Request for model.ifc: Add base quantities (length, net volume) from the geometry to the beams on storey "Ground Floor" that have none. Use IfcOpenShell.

First a look at what the model holds.

```python
import ifcopenshell
import ifcopenshell.util.element
import ifcopenshell.util.unit

model = ifcopenshell.open("model.ifc")
print(model.schema)
for unit_type in ("LENGTHUNIT", "AREAUNIT", "VOLUMEUNIT"):
    print(unit_type, ifcopenshell.util.unit.calculate_unit_scale(model, unit_type))
storey = next(s for s in model.by_type("IfcBuildingStorey") if s.Name == "Ground Floor")
beams = [e for e in ifcopenshell.util.element.get_decomposition(storey) if e.is_a("IfcBeam")]
for e in sorted(beams, key=lambda e: e.id()):
    print(e.id(), e.is_a(), e.Name, list(ifcopenshell.util.element.get_psets(e, qtos_only=True)), sep=" | ")
```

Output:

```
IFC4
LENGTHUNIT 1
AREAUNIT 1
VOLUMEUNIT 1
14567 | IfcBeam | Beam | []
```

```python
import ifcopenshell
import ifcopenshell.api.pset
import ifcopenshell.geom
import ifcopenshell.util.element
import ifcopenshell.util.shape
import ifcopenshell.util.unit

model = ifcopenshell.open("model.ifc")
unit_scale = ifcopenshell.util.unit.calculate_unit_scale(model)
volume_scale = ifcopenshell.util.unit.calculate_unit_scale(model, "VOLUMEUNIT")
settings = ifcopenshell.geom.settings()

storey = next(s for s in model.by_type("IfcBuildingStorey") if s.Name == "Ground Floor")
beams = [e for e in ifcopenshell.util.element.get_decomposition(storey) if e.is_a("IfcBeam")]

for e in sorted(beams, key=lambda e: e.id()):
    if ifcopenshell.util.element.get_psets(e, qtos_only=True, should_inherit=False):
        continue
    # Geometry comes back in metres, in the element's own axes.
    shape = ifcopenshell.geom.create_shape(settings, e)
    values = {
        "Length": ifcopenshell.util.shape.get_max_xyz(shape.geometry) / unit_scale,
        "NetVolume": ifcopenshell.util.shape.get_volume(shape.geometry) / volume_scale,
    }
    qto = ifcopenshell.api.pset.add_qto(model, product=e, name="Qto_BeamBaseQuantities")
    ifcopenshell.api.pset.edit_qto(model, qto=qto, properties=values)
    print(e.id(), {k: round(v, 3) for k, v in values.items()})

model.write("model_v2.ifc")
```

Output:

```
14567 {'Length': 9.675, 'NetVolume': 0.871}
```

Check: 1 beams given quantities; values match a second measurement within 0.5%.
